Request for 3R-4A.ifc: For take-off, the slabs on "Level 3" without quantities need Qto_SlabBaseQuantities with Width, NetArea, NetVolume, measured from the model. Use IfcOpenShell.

First a look at what the model holds.

```python
import ifcopenshell
import ifcopenshell.util.element
import ifcopenshell.util.unit

model = ifcopenshell.open("3R-4A.ifc")
print(model.schema)
for unit_type in ("LENGTHUNIT", "AREAUNIT", "VOLUMEUNIT"):
    print(unit_type, ifcopenshell.util.unit.calculate_unit_scale(model, unit_type))
storey = next(s for s in model.by_type("IfcBuildingStorey") if s.Name == "Level 3")
slabs = [e for e in ifcopenshell.util.element.get_decomposition(storey) if e.is_a("IfcSlab")]
for e in sorted(slabs, key=lambda e: e.id()):
    print(e.id(), e.is_a(), e.Name, list(ifcopenshell.util.element.get_psets(e, qtos_only=True)), sep=" | ")
```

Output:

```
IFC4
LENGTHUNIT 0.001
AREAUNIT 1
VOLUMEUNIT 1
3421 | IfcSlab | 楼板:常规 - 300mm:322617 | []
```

```python
import ifcopenshell
import ifcopenshell.api.pset
import ifcopenshell.geom
import ifcopenshell.util.element
import ifcopenshell.util.shape
import ifcopenshell.util.unit

model = ifcopenshell.open("3R-4A.ifc")
unit_scale = ifcopenshell.util.unit.calculate_unit_scale(model)
area_scale = ifcopenshell.util.unit.calculate_unit_scale(model, "AREAUNIT")
volume_scale = ifcopenshell.util.unit.calculate_unit_scale(model, "VOLUMEUNIT")
settings = ifcopenshell.geom.settings()

storey = next(s for s in model.by_type("IfcBuildingStorey") if s.Name == "Level 3")
slabs = [e for e in ifcopenshell.util.element.get_decomposition(storey) if e.is_a("IfcSlab")]

for e in sorted(slabs, key=lambda e: e.id()):
    if ifcopenshell.util.element.get_psets(e, qtos_only=True, should_inherit=False):
        continue
    # Geometry comes back in metres, in the element's own axes.
    shape = ifcopenshell.geom.create_shape(settings, e)
    values = {
        "Width": ifcopenshell.util.shape.get_z(shape.geometry) / unit_scale,
        "NetArea": ifcopenshell.util.shape.get_footprint_area(shape.geometry) / area_scale,
        "NetVolume": ifcopenshell.util.shape.get_volume(shape.geometry) / volume_scale,
    }
    qto = ifcopenshell.api.pset.add_qto(model, product=e, name="Qto_SlabBaseQuantities")
    ifcopenshell.api.pset.edit_qto(model, qto=qto, properties=values)
    print(e.id(), {k: round(v, 3) for k, v in values.items()})

model.write("3R-4A-out.ifc")
```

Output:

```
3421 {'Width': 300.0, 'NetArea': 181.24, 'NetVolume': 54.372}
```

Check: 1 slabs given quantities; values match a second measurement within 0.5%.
